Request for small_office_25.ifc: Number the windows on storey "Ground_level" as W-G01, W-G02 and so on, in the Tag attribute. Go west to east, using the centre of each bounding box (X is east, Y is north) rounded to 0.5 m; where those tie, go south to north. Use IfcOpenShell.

First a look at what the model holds.

```python
import ifcopenshell
import ifcopenshell.util.element
import ifcopenshell.util.placement

model = ifcopenshell.open("small_office_25.ifc")
print(model.schema)
storey = next(s for s in model.by_type("IfcBuildingStorey") if s.Name == "Ground_level")
windows = [e for e in ifcopenshell.util.element.get_decomposition(storey) if e.is_a("IfcWindow")]
for e in sorted(windows, key=lambda e: e.id()):
    origin = ifcopenshell.util.placement.get_local_placement(e.ObjectPlacement)[:3, 3]
    print(e.id(), e.Tag, e.Name, origin.round(2) + 0.0, sep=" | ")
```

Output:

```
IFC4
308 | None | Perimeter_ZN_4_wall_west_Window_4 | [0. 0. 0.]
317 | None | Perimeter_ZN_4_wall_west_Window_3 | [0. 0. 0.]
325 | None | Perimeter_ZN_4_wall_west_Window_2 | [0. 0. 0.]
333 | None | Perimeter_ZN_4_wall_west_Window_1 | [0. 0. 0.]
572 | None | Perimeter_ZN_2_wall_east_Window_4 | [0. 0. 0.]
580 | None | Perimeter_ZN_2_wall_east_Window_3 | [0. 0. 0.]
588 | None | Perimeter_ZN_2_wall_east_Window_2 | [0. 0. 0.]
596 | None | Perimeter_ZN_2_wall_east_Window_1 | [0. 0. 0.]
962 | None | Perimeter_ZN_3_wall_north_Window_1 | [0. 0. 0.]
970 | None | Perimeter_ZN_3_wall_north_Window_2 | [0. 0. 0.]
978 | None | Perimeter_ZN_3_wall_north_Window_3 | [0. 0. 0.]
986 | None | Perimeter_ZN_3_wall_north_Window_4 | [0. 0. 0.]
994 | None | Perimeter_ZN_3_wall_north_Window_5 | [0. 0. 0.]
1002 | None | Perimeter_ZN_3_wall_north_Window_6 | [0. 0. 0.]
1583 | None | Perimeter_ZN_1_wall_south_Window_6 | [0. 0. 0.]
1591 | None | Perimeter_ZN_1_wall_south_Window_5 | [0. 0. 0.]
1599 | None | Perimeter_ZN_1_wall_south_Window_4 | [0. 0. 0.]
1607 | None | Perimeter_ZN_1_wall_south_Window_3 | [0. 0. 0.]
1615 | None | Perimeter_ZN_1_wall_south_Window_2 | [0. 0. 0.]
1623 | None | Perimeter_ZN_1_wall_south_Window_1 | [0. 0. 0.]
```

```python
import ifcopenshell
import ifcopenshell.geom
import ifcopenshell.util.element
import ifcopenshell.util.shape

model = ifcopenshell.open("small_office_25.ifc")
settings = ifcopenshell.geom.settings()
settings.set("use-world-coords", True)


def centre(element):
    shape = ifcopenshell.geom.create_shape(settings, element)
    return ifcopenshell.util.shape.get_bbox_centroid(shape.geometry)


storey = next(s for s in model.by_type("IfcBuildingStorey") if s.Name == "Ground_level")
windows = [e for e in ifcopenshell.util.element.get_decomposition(storey) if e.is_a("IfcWindow")]

# Insertion points can sit at a corner or the storey origin, so sort by the geometry (in metres).
centres = {e: centre(e) for e in windows}
windows.sort(key=lambda e: (round(centres[e][0] / 0.5), centres[e][1]))

for i, e in enumerate(windows, start=1):
    number = f"W-G{i:02d}"
    e.Tag = number
    print(e.id(), number)

model.write("small_office_25_rev.ifc")
```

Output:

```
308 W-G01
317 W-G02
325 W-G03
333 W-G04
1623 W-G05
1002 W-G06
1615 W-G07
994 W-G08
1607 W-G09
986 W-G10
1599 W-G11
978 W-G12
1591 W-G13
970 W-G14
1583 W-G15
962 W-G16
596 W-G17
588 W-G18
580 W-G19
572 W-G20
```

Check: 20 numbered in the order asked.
